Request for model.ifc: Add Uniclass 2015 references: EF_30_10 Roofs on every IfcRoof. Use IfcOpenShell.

First a look at what the model holds.

```python
import ifcopenshell

model = ifcopenshell.open("model.ifc")
print(model.schema)
print("classifications:", [c.Name for c in model.by_type("IfcClassification")])
for ifc_class in ("IfcDoor", "IfcRoof", "IfcStair", "IfcWall", "IfcWindow"):
    print(ifc_class, len(model.by_type(ifc_class)))
```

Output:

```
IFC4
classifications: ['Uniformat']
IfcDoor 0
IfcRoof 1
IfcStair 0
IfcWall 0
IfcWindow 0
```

```python
import ifcopenshell
import ifcopenshell.api.classification

model = ifcopenshell.open("model.ifc")

system = ifcopenshell.api.classification.add_classification(model, classification="Uniclass 2015")

codes = {
    "IfcRoof": ("EF_30_10", "Roofs"),
}
for ifc_class, (code, name) in codes.items():
    products = model.by_type(ifc_class)
    ifcopenshell.api.classification.add_reference(
        model, products=products, classification=system, identification=code, name=name
    )
    print(code, len(products))

model.write("model-out.ifc")
```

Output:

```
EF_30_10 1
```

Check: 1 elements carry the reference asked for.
